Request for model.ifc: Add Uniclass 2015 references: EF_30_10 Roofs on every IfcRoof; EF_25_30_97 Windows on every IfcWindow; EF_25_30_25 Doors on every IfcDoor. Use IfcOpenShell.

First a look at what the model holds.

```python
import ifcopenshell

model = ifcopenshell.open("model.ifc")
print(model.schema)
print("classifications:", [c.Name for c in model.by_type("IfcClassification")])
for ifc_class in ("IfcDoor", "IfcRoof", "IfcStair", "IfcWall", "IfcWindow"):
    print(ifc_class, len(model.by_type(ifc_class)))
```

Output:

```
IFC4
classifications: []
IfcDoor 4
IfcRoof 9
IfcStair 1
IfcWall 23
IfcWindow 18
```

```python
import ifcopenshell
import ifcopenshell.api.classification

model = ifcopenshell.open("model.ifc")

system = ifcopenshell.api.classification.add_classification(model, classification="Uniclass 2015")

codes = {
    "IfcRoof": ("EF_30_10", "Roofs"),
    "IfcWindow": ("EF_25_30_97", "Windows"),
    "IfcDoor": ("EF_25_30_25", "Doors"),
}
for ifc_class, (code, name) in codes.items():
    products = model.by_type(ifc_class)
    ifcopenshell.api.classification.add_reference(
        model, products=products, classification=system, identification=code, name=name
    )
    print(code, len(products))

model.write("model_updated.ifc")
```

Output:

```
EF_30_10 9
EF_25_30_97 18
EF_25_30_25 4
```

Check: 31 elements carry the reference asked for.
